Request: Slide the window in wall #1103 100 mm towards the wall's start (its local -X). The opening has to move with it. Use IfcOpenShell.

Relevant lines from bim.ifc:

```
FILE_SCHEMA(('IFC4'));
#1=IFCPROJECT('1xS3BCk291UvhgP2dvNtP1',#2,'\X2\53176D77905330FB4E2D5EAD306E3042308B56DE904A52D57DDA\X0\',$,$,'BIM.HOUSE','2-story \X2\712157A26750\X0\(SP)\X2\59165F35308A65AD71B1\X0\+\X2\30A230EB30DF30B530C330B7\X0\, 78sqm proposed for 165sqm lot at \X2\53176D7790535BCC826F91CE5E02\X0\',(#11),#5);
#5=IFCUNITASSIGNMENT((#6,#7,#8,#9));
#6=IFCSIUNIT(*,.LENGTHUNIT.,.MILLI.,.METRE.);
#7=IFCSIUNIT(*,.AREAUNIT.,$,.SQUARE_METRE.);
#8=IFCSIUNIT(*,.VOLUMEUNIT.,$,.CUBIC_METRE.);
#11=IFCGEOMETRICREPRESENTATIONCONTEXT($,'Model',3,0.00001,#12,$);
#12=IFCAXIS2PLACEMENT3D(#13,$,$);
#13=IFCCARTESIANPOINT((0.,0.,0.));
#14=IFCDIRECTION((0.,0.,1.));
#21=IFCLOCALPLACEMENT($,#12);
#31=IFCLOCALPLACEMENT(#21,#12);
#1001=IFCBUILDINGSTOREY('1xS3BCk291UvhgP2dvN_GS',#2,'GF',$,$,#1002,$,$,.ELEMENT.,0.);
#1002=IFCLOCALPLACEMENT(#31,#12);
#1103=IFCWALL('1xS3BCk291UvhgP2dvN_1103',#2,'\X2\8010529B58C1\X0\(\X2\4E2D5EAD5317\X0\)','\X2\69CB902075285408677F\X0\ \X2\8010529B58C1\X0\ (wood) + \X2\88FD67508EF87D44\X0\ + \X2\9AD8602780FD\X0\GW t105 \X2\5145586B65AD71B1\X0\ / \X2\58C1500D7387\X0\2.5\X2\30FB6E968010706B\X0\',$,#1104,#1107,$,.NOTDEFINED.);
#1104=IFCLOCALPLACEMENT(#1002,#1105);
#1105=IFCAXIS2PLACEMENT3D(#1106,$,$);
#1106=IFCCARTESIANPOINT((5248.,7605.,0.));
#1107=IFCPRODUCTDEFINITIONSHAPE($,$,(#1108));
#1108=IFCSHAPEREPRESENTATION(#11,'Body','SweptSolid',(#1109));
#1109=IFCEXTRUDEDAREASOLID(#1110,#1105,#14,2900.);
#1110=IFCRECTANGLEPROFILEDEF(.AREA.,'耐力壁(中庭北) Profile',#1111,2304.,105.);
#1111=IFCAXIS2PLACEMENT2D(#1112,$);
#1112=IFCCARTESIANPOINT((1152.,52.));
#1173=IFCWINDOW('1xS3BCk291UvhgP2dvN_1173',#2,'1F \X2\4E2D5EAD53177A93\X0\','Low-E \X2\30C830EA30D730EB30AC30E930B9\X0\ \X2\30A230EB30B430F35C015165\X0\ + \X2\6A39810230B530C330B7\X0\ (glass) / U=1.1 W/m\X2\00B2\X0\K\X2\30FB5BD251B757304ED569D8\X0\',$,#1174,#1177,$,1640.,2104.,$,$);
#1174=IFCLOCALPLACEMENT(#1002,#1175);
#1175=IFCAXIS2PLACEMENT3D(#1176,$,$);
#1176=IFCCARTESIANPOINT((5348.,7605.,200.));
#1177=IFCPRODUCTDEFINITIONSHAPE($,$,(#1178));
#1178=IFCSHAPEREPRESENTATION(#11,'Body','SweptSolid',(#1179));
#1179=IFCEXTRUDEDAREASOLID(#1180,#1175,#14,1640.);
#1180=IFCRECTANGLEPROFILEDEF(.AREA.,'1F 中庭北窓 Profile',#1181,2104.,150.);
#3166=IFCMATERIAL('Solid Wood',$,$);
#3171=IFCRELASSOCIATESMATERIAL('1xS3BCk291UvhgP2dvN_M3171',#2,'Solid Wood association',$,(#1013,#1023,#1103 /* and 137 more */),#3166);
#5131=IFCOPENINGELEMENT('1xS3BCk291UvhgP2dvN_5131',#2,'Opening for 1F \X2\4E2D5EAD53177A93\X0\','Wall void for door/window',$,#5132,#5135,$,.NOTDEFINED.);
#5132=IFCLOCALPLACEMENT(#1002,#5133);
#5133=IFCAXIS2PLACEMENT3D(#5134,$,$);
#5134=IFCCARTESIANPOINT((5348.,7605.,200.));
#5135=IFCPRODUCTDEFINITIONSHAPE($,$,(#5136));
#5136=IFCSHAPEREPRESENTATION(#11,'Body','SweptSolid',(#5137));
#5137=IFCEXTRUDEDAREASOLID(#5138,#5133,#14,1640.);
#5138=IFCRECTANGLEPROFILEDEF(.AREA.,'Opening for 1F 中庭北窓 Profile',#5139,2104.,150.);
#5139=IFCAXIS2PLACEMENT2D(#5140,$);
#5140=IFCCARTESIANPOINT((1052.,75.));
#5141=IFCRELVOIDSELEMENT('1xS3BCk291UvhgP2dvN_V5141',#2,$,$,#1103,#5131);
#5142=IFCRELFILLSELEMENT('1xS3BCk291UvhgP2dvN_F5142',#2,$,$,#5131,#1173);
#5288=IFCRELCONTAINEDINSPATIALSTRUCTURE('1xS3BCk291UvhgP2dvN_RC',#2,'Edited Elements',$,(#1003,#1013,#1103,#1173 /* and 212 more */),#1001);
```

```python
import ifcopenshell
import ifcopenshell.api.geometry
import ifcopenshell.util.placement

model = ifcopenshell.open("bim.ifc")

window = model.by_guid("1xS3BCk291UvhgP2dvN_1173")
opening = window.FillsVoids[0].RelatingOpeningElement
wall = opening.VoidsElements[0].RelatingBuildingElement

wall_matrix = ifcopenshell.util.placement.get_local_placement(wall.ObjectPlacement)
shift = wall_matrix[:3, 0] * -100.0
before = ifcopenshell.util.placement.get_local_placement(window.ObjectPlacement)[:3, 3].copy()

# The window is not placed relative to its opening, so move both.
for product in (opening, window):
    matrix = ifcopenshell.util.placement.get_local_placement(product.ObjectPlacement)
    matrix[:3, 3] += shift
    ifcopenshell.api.geometry.edit_object_placement(model, product=product, matrix=matrix, is_si=False)

after = ifcopenshell.util.placement.get_local_placement(window.ObjectPlacement)[:3, 3]
print("window moved by", (after - before).round(3) + 0.0)

model.write("bim_edited.ifc")
```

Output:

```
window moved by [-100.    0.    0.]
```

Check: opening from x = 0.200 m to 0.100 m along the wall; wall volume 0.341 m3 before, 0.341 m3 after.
